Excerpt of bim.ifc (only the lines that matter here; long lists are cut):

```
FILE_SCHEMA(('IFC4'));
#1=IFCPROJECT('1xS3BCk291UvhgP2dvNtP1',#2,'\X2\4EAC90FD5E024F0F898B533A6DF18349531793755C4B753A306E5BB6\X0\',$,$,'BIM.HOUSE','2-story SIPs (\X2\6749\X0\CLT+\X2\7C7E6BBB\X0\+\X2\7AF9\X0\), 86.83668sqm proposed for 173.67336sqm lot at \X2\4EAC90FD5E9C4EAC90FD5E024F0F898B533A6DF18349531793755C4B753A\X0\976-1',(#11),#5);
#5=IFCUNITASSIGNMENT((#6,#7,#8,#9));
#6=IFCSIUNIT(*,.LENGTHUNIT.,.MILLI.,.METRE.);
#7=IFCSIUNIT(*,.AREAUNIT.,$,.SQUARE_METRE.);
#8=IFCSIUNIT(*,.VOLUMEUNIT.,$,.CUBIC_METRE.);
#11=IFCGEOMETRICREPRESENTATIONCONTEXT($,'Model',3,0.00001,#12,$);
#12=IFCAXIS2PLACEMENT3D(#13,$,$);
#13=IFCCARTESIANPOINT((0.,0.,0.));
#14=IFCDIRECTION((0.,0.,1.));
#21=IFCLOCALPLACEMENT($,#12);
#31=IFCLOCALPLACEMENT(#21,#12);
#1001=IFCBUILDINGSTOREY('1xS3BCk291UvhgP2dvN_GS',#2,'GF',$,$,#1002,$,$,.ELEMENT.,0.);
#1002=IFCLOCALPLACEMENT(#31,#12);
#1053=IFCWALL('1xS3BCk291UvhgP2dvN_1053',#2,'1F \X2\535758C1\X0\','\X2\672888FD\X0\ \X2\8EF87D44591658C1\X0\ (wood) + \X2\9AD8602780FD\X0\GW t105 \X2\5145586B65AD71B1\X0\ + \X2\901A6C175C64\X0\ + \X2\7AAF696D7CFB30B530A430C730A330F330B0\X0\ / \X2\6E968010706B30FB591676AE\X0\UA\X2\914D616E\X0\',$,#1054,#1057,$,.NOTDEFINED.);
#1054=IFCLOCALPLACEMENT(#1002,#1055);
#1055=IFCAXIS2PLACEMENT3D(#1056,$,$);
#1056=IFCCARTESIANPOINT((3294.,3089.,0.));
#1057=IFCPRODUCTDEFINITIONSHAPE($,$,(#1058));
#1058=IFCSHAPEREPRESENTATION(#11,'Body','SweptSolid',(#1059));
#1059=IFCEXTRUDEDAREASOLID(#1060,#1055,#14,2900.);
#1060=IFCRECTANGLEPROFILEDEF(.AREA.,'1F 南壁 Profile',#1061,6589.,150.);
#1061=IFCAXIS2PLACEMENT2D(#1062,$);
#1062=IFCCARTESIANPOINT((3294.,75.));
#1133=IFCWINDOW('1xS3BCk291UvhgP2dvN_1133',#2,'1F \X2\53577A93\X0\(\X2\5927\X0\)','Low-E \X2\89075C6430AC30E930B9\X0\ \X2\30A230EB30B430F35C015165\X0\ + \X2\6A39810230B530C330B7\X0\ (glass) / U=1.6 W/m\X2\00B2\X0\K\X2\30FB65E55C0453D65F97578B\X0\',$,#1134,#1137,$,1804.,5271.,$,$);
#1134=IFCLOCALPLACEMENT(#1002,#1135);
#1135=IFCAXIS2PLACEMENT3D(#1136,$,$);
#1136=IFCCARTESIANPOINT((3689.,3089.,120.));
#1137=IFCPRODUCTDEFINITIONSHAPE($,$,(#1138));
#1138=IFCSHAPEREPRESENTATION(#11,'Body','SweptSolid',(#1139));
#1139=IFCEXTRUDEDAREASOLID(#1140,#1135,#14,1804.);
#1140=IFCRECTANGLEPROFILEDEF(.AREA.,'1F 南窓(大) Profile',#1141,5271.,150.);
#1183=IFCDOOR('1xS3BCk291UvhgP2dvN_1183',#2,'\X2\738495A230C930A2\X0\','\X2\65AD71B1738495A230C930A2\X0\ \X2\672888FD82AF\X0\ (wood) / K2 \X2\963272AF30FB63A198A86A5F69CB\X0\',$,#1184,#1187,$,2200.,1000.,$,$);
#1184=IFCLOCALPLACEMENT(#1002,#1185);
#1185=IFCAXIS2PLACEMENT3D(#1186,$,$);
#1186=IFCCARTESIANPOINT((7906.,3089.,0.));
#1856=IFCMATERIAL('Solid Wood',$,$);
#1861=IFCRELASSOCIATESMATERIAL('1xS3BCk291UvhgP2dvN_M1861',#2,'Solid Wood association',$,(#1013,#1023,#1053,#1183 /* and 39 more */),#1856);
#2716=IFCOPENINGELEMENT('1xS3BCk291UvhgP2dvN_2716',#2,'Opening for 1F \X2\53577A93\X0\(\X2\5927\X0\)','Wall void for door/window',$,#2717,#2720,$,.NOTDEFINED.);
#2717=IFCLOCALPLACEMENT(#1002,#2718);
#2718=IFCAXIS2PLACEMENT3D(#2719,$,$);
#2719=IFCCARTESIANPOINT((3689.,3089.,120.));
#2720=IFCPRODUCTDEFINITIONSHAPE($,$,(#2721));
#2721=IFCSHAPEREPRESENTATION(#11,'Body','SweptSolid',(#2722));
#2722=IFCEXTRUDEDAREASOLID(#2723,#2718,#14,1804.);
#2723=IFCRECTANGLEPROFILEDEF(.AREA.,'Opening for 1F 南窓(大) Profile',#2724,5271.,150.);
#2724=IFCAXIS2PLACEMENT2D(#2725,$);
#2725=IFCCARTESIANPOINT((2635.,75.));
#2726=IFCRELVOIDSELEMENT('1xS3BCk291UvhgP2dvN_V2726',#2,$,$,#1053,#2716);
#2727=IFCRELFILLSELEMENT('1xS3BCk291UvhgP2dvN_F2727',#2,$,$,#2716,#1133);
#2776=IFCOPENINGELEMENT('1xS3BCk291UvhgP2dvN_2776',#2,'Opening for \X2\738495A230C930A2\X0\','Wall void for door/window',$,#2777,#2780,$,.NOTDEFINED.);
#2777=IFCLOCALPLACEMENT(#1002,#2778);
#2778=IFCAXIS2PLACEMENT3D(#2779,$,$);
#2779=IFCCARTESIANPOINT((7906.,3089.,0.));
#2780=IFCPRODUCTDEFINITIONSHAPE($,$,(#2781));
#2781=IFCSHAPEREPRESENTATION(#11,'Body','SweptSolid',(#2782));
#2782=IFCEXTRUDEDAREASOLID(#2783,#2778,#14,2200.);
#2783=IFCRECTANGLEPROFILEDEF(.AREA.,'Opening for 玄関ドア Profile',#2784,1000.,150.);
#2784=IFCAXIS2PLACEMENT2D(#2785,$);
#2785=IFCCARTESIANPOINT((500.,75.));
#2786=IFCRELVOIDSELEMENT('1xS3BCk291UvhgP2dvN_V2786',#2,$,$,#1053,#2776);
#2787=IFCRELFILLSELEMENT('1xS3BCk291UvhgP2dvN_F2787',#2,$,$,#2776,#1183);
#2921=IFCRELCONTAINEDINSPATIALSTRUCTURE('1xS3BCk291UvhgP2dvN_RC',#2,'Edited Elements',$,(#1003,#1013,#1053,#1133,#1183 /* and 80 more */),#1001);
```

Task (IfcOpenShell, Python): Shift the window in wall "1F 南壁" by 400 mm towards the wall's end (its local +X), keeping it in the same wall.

```python
import ifcopenshell
import ifcopenshell.api.geometry
import ifcopenshell.util.placement
import ifcopenshell.util.unit

model = ifcopenshell.open("bim.ifc")
unit_scale = ifcopenshell.util.unit.calculate_unit_scale(model)

window = model.by_guid("1xS3BCk291UvhgP2dvN_1133")
opening = window.FillsVoids[0].RelatingOpeningElement
wall = opening.VoidsElements[0].RelatingBuildingElement

wall_matrix = ifcopenshell.util.placement.get_local_placement(wall.ObjectPlacement)
shift = wall_matrix[:3, 0] * 0.4 / unit_scale
before = ifcopenshell.util.placement.get_local_placement(window.ObjectPlacement)[:3, 3].copy()

# The window is not placed relative to its opening, so move both.
for product in (opening, window):
    matrix = ifcopenshell.util.placement.get_local_placement(product.ObjectPlacement)
    matrix[:3, 3] += shift
    ifcopenshell.api.geometry.edit_object_placement(model, product=product, matrix=matrix, is_si=False)

after = ifcopenshell.util.placement.get_local_placement(window.ObjectPlacement)[:3, 3]
print("window moved by", (after - before).round(3) + 0.0)

model.write("bim_updated.ifc")
```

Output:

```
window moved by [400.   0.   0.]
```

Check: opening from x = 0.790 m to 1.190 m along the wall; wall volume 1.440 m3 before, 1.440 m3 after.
